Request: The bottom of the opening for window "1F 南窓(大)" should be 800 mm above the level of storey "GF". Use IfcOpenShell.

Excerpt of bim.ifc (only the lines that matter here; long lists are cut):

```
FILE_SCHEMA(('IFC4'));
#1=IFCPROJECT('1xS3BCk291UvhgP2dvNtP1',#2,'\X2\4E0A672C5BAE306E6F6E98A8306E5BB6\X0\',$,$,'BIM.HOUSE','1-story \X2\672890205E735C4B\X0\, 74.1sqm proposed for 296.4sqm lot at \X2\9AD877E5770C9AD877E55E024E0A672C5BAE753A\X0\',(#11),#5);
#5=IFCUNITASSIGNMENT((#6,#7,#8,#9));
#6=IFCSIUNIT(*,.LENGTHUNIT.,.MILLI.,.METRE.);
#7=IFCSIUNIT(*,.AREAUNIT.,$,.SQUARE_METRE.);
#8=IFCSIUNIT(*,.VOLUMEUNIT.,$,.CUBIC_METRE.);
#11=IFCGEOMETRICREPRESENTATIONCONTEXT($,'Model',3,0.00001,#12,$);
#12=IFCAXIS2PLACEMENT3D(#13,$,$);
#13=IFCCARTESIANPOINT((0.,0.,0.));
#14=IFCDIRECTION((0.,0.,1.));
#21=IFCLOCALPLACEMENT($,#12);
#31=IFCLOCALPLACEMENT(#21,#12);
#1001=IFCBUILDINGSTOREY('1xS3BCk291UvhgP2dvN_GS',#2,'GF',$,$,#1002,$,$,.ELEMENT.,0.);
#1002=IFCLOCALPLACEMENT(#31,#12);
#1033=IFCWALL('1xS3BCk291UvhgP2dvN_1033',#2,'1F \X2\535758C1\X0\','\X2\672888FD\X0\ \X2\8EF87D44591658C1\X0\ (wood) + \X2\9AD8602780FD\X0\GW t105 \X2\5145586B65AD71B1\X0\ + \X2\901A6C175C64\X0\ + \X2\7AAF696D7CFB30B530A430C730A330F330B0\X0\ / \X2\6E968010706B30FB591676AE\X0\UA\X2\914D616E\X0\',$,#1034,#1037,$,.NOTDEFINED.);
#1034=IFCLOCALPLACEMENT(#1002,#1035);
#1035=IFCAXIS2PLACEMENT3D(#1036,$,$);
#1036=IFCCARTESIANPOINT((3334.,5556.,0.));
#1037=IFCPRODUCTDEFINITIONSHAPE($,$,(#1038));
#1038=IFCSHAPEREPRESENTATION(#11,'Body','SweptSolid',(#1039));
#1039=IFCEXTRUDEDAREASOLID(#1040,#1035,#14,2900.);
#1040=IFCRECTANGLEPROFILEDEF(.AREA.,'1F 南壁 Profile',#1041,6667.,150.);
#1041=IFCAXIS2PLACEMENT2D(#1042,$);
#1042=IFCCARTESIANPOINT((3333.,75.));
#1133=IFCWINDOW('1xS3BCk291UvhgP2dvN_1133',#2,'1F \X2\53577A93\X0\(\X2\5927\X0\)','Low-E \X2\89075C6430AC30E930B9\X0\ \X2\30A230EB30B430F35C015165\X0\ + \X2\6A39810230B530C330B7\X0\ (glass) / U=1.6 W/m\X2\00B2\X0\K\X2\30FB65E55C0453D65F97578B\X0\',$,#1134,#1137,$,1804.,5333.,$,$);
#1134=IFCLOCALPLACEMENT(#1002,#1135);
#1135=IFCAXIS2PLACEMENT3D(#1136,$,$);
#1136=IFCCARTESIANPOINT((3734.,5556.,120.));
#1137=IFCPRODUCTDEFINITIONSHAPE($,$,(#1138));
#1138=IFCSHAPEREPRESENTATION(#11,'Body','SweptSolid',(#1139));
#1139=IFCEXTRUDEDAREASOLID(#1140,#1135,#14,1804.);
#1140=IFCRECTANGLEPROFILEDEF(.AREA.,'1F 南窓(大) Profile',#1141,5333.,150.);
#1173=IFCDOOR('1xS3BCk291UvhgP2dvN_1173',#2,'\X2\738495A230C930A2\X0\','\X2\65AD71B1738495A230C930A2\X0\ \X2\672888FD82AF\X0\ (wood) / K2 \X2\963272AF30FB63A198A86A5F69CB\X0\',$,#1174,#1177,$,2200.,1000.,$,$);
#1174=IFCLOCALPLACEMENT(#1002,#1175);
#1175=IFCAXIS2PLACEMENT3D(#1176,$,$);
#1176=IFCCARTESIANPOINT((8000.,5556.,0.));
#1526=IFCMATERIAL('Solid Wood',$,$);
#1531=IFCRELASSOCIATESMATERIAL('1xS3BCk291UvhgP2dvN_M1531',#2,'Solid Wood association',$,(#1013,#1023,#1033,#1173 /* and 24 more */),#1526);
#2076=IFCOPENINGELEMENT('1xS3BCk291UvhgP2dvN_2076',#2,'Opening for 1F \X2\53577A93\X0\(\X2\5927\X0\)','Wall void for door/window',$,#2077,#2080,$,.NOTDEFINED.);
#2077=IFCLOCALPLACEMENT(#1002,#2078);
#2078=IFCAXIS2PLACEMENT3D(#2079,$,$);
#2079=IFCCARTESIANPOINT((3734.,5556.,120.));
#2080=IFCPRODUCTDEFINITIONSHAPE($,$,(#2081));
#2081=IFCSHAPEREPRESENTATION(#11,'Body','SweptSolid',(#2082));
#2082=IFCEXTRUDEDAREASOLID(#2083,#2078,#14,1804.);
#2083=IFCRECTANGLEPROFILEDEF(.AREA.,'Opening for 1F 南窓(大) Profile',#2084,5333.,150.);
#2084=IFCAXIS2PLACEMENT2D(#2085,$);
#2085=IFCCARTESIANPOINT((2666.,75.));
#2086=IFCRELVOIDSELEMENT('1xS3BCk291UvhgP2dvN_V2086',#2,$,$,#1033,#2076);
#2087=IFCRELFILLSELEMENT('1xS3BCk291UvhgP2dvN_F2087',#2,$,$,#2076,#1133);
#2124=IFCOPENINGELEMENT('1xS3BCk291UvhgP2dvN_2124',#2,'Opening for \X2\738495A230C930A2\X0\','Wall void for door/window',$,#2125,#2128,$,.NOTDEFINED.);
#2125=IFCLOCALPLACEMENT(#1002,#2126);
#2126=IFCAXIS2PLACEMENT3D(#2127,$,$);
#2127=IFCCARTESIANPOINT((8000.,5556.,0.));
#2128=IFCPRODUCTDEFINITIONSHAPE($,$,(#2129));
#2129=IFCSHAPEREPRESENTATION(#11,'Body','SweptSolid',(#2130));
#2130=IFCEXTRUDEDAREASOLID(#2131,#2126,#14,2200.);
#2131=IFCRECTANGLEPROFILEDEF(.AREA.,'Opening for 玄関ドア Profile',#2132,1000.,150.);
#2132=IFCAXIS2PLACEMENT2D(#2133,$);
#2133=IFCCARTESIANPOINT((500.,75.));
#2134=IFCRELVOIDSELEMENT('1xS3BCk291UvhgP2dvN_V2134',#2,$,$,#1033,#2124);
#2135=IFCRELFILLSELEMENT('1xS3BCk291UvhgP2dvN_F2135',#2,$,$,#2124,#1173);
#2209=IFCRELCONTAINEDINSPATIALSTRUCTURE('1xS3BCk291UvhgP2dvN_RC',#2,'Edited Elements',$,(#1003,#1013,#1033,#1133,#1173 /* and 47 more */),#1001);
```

```python
import numpy as np
import ifcopenshell
import ifcopenshell.api.geometry
import ifcopenshell.geom
import ifcopenshell.util.element
import ifcopenshell.util.placement
import ifcopenshell.util.shape
import ifcopenshell.util.unit

model = ifcopenshell.open("bim.ifc")
unit_scale = ifcopenshell.util.unit.calculate_unit_scale(model)

window = model.by_guid("1xS3BCk291UvhgP2dvN_1133")
opening = window.FillsVoids[0].RelatingOpeningElement
storey = ifcopenshell.util.element.get_container(window, ifc_class="IfcBuildingStorey")
level = ifcopenshell.util.placement.get_local_placement(storey.ObjectPlacement)[2, 3]

# The opening's origin need not be at the sill, so measure its lowest point.
shape = ifcopenshell.geom.create_shape(ifcopenshell.geom.settings(), opening)
bottom = ifcopenshell.util.shape.get_shape_bottom_elevation(shape, shape.geometry) / unit_scale
dz = level + 800.0 - bottom

shift = np.array([0.0, 0.0, dz])
# The window is not placed relative to its opening, so move both.
for product in (opening, window):
    matrix = ifcopenshell.util.placement.get_local_placement(product.ObjectPlacement)
    matrix[:3, 3] += shift
    ifcopenshell.api.geometry.edit_object_placement(model, product=product, matrix=matrix, is_si=False)

print(f"moved by {dz * unit_scale:+.3f} m")

model.write("bim_v2.ifc")
```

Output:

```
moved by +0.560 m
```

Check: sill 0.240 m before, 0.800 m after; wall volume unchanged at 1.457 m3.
